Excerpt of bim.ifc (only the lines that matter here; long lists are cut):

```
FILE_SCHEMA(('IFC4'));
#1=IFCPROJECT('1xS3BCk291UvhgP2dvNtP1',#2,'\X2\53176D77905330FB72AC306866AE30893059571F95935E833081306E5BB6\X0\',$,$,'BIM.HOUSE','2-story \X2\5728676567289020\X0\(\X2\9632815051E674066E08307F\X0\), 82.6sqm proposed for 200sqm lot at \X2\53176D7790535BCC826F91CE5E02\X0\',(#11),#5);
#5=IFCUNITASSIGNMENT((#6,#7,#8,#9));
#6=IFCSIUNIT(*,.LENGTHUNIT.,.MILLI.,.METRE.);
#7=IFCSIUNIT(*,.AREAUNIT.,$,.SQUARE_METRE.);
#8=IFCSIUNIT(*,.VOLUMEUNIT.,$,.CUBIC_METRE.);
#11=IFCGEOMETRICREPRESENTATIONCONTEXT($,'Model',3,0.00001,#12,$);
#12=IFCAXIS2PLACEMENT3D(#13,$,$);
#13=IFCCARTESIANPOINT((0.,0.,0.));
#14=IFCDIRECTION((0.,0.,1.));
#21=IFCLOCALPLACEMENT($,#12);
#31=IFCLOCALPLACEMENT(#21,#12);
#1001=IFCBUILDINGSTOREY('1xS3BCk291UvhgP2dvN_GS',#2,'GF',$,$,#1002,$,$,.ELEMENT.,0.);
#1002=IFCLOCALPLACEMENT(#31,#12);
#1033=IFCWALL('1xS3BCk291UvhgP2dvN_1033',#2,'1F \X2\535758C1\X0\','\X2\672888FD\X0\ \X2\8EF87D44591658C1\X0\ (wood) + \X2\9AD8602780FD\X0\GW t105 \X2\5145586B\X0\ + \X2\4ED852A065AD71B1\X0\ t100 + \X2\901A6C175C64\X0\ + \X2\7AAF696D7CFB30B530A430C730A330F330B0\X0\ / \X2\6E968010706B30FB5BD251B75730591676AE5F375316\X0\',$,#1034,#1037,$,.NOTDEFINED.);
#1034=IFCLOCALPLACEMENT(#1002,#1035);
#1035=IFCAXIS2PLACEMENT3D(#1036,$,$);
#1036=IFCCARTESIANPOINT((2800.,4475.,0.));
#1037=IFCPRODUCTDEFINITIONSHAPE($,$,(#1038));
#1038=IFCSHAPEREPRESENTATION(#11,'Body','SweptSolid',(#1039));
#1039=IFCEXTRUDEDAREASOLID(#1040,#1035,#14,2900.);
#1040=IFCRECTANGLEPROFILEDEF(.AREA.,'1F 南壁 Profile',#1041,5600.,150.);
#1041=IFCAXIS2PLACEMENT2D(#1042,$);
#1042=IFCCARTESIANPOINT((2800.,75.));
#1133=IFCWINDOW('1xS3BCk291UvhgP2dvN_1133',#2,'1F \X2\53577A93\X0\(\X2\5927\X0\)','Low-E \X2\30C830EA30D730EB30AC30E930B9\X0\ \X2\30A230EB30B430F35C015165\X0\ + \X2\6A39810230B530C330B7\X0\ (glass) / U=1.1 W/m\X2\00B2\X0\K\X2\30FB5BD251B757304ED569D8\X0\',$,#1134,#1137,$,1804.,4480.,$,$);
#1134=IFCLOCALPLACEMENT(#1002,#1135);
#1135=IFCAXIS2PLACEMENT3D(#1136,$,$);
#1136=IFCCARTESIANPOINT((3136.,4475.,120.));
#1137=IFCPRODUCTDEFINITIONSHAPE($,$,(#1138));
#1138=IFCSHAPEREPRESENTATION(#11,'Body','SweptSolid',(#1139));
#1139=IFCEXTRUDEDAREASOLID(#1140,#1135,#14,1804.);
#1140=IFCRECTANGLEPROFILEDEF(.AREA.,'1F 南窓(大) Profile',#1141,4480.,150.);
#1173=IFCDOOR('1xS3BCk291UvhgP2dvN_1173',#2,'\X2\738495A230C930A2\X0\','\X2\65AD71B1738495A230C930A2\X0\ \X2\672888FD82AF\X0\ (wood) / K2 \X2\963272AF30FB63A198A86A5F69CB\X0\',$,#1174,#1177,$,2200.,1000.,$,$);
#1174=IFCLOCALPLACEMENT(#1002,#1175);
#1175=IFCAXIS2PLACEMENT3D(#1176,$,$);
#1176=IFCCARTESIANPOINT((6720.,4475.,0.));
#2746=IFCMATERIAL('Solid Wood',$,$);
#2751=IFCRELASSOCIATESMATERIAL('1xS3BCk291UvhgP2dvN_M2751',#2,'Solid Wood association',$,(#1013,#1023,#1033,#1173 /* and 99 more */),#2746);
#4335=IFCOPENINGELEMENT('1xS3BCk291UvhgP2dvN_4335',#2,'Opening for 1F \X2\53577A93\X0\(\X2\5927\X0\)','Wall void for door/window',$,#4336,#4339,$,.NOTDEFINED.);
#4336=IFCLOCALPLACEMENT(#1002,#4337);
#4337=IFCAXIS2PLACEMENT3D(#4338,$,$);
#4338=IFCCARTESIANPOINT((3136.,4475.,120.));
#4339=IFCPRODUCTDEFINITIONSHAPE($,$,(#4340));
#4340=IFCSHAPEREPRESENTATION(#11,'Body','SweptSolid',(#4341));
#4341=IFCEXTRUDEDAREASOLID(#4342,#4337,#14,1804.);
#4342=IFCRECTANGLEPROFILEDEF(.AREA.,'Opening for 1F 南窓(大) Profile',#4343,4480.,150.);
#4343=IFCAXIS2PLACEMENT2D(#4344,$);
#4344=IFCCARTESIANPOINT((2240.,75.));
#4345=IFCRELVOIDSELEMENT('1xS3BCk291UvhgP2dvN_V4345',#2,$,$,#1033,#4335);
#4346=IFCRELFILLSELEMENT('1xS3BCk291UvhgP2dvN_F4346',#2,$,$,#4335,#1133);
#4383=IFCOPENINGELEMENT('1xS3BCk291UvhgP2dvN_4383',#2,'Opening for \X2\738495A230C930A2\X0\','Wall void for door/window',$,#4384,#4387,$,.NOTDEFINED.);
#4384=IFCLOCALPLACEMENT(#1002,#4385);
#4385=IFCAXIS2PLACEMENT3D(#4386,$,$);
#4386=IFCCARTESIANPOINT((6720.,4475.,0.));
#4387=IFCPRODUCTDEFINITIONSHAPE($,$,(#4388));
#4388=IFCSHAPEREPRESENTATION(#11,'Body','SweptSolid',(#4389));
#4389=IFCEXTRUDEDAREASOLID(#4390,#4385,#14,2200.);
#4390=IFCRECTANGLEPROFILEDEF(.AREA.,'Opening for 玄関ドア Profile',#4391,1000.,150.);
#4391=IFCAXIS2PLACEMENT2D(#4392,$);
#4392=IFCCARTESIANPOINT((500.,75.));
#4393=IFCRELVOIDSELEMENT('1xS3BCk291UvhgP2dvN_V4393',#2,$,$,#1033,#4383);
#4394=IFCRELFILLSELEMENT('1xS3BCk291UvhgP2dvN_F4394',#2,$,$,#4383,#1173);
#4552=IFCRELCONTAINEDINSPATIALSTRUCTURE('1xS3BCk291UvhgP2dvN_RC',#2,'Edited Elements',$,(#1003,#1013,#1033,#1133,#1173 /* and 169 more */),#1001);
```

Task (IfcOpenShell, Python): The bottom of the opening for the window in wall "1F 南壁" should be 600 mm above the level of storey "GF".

```python
import numpy as np
import ifcopenshell
import ifcopenshell.api.geometry
import ifcopenshell.geom
import ifcopenshell.util.element
import ifcopenshell.util.placement
import ifcopenshell.util.shape
import ifcopenshell.util.unit

model = ifcopenshell.open("bim.ifc")
unit_scale = ifcopenshell.util.unit.calculate_unit_scale(model)

window = model.by_id(1133)
opening = window.FillsVoids[0].RelatingOpeningElement
storey = ifcopenshell.util.element.get_container(window, ifc_class="IfcBuildingStorey")
level = ifcopenshell.util.placement.get_local_placement(storey.ObjectPlacement)[2, 3]

# The opening's origin need not be at the sill, so measure its lowest point.
shape = ifcopenshell.geom.create_shape(ifcopenshell.geom.settings(), opening)
bottom = ifcopenshell.util.shape.get_shape_bottom_elevation(shape, shape.geometry) / unit_scale
dz = level + 0.6 / unit_scale - bottom

shift = np.array([0.0, 0.0, dz])
# The window is not placed relative to its opening, so move both.
for product in (opening, window):
    matrix = ifcopenshell.util.placement.get_local_placement(product.ObjectPlacement)
    matrix[:3, 3] += shift
    ifcopenshell.api.geometry.edit_object_placement(model, product=product, matrix=matrix, is_si=False)

print(f"moved by {dz * unit_scale:+.3f} m")

model.write("bim_updated.ifc")
```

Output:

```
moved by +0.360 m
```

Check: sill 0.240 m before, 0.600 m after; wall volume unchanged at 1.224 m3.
